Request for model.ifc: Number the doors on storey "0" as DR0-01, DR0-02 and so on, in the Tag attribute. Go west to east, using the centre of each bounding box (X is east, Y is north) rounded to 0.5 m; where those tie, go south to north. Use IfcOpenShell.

First a look at what the model holds.

```python
import ifcopenshell
import ifcopenshell.util.element
import ifcopenshell.util.placement

model = ifcopenshell.open("model.ifc")
print(model.schema)
storey = next(s for s in model.by_type("IfcBuildingStorey") if s.Name == "0")
doors = [e for e in ifcopenshell.util.element.get_decomposition(storey) if e.is_a("IfcDoor")]
for e in sorted(doors, key=lambda e: e.id()):
    origin = ifcopenshell.util.placement.get_local_placement(e.ObjectPlacement)[:3, 3]
    print(e.id(), e.Tag, e.Name, origin.round(2) + 0.0, sep=" | ")
```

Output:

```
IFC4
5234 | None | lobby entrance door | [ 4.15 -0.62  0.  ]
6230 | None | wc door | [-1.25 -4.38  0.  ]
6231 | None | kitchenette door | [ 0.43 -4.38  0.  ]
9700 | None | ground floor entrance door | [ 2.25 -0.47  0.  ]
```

```python
import ifcopenshell
import ifcopenshell.geom
import ifcopenshell.util.element
import ifcopenshell.util.shape

model = ifcopenshell.open("model.ifc")
settings = ifcopenshell.geom.settings()
settings.set("use-world-coords", True)


def centre(element):
    shape = ifcopenshell.geom.create_shape(settings, element)
    return ifcopenshell.util.shape.get_bbox_centroid(shape.geometry)


storey = next(s for s in model.by_type("IfcBuildingStorey") if s.Name == "0")
doors = [e for e in ifcopenshell.util.element.get_decomposition(storey) if e.is_a("IfcDoor")]

# Insertion points can sit at a corner or the storey origin, so sort by the geometry (in metres).
centres = {e: centre(e) for e in doors}
doors.sort(key=lambda e: (round(centres[e][0] / 0.5), centres[e][1]))

for i, e in enumerate(doors, start=1):
    number = f"DR0-{i:02d}"
    e.Tag = number
    print(e.id(), number)

model.write("model_edited.ifc")
```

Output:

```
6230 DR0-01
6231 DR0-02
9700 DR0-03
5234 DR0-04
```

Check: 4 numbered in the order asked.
